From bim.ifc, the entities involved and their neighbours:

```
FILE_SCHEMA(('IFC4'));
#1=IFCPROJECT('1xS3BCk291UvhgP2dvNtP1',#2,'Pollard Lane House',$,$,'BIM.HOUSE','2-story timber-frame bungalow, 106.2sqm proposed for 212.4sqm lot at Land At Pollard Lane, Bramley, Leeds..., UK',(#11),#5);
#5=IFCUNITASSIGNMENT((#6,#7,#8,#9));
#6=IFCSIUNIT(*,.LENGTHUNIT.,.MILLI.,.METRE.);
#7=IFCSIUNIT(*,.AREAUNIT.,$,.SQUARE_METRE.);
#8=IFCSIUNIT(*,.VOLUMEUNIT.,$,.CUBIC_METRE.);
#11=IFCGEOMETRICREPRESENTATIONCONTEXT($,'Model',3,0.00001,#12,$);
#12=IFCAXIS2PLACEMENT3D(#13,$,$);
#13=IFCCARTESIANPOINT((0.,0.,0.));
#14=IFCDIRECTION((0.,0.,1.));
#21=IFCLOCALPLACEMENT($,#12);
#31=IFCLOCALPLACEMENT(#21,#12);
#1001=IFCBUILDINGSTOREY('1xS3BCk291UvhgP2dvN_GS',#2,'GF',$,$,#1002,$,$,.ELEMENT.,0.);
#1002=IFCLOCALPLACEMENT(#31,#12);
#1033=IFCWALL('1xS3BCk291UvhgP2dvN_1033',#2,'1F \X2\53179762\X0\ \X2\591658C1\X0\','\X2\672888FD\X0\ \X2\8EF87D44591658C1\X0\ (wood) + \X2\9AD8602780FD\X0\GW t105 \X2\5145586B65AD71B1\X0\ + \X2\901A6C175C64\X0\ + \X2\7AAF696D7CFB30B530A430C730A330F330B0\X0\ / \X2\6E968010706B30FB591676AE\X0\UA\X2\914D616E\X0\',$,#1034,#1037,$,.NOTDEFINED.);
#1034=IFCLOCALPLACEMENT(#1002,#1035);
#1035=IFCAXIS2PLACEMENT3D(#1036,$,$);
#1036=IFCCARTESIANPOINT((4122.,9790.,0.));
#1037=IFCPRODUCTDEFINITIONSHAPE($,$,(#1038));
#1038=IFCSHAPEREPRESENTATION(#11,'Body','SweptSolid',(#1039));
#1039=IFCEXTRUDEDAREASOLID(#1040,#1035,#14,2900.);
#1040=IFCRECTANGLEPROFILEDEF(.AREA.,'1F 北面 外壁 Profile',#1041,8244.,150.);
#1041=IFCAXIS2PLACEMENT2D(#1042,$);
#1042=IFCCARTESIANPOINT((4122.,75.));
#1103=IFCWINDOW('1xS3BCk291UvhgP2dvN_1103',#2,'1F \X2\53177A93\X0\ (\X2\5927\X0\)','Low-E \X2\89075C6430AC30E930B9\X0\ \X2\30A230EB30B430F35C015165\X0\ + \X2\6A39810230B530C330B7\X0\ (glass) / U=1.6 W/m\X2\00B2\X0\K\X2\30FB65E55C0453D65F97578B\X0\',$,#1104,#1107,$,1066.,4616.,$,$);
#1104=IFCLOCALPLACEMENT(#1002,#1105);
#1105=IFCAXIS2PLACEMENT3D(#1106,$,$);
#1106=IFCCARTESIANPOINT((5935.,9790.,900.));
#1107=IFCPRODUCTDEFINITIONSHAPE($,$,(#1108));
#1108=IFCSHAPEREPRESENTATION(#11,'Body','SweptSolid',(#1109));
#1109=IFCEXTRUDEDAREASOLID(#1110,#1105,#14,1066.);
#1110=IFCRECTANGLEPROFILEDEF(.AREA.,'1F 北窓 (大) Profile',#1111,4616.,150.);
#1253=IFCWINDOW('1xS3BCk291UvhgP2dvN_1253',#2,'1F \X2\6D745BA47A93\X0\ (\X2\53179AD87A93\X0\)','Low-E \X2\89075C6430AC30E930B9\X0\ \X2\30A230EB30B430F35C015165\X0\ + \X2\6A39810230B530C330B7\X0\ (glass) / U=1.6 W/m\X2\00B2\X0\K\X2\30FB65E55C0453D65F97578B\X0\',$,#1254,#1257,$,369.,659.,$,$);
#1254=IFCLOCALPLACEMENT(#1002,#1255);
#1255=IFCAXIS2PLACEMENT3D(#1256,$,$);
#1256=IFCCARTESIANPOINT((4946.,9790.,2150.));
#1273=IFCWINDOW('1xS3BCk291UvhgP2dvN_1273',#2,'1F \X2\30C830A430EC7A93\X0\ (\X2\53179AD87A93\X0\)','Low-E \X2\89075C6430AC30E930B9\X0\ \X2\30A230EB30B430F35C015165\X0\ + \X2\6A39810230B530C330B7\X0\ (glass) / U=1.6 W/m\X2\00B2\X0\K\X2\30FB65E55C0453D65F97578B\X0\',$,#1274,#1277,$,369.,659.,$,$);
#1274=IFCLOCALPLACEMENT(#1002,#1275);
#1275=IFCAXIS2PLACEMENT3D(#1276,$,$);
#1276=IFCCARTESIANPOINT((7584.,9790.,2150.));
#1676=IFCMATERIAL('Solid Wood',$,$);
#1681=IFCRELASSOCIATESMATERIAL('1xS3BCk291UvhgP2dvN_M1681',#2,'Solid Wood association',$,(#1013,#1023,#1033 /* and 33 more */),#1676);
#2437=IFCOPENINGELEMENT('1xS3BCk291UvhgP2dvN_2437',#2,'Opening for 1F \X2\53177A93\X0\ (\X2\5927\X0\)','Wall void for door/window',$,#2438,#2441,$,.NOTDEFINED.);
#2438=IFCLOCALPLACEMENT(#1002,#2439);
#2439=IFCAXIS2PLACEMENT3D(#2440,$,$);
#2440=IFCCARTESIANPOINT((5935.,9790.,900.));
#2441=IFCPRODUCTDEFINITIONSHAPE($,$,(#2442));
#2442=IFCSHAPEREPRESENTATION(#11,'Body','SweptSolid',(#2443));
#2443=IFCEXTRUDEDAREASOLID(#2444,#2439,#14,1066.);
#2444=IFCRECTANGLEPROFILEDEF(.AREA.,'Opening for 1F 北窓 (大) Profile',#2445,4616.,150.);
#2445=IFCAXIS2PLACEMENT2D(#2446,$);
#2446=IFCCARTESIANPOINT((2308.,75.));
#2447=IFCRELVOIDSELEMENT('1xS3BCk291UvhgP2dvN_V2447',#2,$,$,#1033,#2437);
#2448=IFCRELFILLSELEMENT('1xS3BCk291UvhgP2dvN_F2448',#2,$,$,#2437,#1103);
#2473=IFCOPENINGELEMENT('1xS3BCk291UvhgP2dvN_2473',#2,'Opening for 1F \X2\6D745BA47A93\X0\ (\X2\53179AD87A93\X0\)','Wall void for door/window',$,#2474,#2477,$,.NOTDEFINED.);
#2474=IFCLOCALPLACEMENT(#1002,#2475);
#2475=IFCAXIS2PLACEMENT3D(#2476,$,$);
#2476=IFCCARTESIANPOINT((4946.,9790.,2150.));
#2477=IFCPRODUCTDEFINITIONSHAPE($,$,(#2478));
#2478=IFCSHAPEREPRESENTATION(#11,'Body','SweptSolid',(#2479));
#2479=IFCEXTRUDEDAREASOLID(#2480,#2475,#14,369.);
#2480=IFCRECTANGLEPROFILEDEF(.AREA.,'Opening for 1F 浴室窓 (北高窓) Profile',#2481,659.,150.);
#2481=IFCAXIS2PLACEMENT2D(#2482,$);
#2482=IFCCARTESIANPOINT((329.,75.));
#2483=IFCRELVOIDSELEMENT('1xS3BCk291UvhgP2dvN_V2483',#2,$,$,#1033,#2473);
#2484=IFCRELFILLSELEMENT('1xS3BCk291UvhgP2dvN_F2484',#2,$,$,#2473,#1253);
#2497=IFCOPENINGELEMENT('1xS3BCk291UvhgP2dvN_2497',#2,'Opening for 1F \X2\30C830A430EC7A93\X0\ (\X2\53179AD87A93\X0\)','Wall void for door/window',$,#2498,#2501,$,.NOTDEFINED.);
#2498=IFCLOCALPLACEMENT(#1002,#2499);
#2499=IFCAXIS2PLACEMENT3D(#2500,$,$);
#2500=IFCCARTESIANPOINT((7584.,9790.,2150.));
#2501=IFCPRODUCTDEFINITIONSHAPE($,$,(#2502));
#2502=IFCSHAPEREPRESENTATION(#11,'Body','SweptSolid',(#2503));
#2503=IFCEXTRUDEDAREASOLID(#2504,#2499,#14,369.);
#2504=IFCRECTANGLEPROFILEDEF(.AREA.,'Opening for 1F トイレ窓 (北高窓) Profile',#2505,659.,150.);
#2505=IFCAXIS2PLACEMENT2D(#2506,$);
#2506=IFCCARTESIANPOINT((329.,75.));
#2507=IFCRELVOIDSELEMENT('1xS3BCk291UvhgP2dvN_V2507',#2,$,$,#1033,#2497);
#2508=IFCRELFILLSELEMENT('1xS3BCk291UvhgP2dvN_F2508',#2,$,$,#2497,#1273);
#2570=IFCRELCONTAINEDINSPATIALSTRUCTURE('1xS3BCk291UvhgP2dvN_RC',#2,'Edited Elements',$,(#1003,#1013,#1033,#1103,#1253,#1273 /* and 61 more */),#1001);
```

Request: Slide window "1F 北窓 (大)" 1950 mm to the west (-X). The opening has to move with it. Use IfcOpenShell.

```python
import ifcopenshell
import ifcopenshell.api.geometry
import ifcopenshell.util.placement

model = ifcopenshell.open("bim.ifc")

window = model.by_id(1103)
opening = window.FillsVoids[0].RelatingOpeningElement
wall = opening.VoidsElements[0].RelatingBuildingElement

wall_matrix = ifcopenshell.util.placement.get_local_placement(wall.ObjectPlacement)
shift = wall_matrix[:3, 0] * -1950.0
before = ifcopenshell.util.placement.get_local_placement(window.ObjectPlacement)[:3, 3].copy()

# The window is not placed relative to its opening, so move both.
for product in (opening, window):
    matrix = ifcopenshell.util.placement.get_local_placement(product.ObjectPlacement)
    matrix[:3, 3] += shift
    ifcopenshell.api.geometry.edit_object_placement(model, product=product, matrix=matrix, is_si=False)

after = ifcopenshell.util.placement.get_local_placement(window.ObjectPlacement)[:3, 3]
print("window moved by", (after - before).round(3) + 0.0)

model.write("bim_rev.ifc")
```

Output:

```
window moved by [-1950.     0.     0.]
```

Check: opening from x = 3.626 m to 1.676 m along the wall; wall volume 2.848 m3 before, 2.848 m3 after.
